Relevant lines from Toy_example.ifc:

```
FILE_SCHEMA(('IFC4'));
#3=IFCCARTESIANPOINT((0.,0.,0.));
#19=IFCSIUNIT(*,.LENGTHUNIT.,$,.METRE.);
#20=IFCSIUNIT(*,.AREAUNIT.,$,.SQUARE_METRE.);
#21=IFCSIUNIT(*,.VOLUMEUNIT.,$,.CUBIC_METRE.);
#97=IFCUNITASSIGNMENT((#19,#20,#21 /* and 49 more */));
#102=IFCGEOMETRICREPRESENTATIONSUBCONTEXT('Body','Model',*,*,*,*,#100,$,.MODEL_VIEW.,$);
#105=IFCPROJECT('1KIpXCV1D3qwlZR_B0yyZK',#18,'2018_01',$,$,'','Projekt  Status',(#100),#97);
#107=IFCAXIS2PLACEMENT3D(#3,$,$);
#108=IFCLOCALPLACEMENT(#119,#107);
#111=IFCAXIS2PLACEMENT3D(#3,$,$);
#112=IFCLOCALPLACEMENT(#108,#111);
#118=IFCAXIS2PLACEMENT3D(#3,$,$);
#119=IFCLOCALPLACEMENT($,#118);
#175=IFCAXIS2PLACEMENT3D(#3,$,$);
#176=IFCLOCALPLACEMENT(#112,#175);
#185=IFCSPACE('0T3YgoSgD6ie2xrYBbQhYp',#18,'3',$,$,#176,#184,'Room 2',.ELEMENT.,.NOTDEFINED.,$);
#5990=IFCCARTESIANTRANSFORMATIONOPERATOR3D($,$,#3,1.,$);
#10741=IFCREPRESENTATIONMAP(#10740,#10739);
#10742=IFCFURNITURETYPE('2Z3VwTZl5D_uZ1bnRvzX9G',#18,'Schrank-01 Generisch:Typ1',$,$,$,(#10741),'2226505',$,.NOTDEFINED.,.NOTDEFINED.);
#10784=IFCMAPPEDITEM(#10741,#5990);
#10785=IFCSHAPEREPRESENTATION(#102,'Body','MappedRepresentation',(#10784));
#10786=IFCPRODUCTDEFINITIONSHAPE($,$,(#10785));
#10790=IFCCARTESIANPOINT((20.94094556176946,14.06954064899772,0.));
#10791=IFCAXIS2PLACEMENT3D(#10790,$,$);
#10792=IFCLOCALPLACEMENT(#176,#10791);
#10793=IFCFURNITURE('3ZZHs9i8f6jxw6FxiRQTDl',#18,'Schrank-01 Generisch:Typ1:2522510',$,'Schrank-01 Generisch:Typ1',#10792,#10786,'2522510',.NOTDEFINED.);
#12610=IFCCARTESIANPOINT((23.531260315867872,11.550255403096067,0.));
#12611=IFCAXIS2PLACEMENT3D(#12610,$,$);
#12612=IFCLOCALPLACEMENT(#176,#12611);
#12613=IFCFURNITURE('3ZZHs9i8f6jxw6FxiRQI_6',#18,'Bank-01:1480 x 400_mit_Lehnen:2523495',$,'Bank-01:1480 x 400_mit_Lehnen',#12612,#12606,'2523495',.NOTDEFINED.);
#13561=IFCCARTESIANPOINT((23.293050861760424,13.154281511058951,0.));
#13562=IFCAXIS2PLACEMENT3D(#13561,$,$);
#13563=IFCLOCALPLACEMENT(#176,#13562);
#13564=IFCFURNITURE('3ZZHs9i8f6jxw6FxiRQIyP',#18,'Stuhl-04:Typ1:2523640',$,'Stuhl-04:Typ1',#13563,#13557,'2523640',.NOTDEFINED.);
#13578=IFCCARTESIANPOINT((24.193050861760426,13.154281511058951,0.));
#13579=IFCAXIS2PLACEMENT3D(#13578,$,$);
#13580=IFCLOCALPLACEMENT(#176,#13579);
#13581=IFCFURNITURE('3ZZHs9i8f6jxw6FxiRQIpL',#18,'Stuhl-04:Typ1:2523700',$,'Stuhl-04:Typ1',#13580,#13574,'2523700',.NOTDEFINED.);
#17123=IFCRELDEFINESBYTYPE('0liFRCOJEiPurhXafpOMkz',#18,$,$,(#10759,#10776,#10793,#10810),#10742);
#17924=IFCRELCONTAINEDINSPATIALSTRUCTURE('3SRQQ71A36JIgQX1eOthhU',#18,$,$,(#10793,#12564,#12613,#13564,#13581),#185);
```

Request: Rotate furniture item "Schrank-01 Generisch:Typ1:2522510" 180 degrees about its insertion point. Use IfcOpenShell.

```python
import ifcopenshell
import ifcopenshell.api.geometry
import ifcopenshell.util.placement

model = ifcopenshell.open("Toy_example.ifc")

item = model.by_guid("3ZZHs9i8f6jxw6FxiRQTDl")
matrix = ifcopenshell.util.placement.get_local_placement(item.ObjectPlacement)
matrix = matrix @ ifcopenshell.util.placement.rotation(180, "Z")
ifcopenshell.api.geometry.edit_object_placement(model, product=item, matrix=matrix, is_si=False)

print(ifcopenshell.util.placement.get_local_placement(item.ObjectPlacement).round(3) + 0.0)

model.write("Toy_example_rev.ifc")
```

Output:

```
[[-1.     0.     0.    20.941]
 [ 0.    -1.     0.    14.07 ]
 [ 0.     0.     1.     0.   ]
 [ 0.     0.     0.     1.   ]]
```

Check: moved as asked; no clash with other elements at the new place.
